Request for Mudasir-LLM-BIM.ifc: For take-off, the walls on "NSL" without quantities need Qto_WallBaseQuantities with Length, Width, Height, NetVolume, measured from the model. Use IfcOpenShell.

First a look at what the model holds.

```python
import ifcopenshell
import ifcopenshell.util.element
import ifcopenshell.util.unit

model = ifcopenshell.open("Mudasir-LLM-BIM.ifc")
print(model.schema)
for unit_type in ("LENGTHUNIT", "AREAUNIT", "VOLUMEUNIT"):
    print(unit_type, ifcopenshell.util.unit.calculate_unit_scale(model, unit_type))
storey = next(s for s in model.by_type("IfcBuildingStorey") if s.Name == "NSL")
walls = [e for e in ifcopenshell.util.element.get_decomposition(storey) if e.is_a("IfcWall")]
for e in sorted(walls, key=lambda e: e.id()):
    print(e.id(), e.is_a(), e.Name, list(ifcopenshell.util.element.get_psets(e, qtos_only=True)), sep=" | ")
```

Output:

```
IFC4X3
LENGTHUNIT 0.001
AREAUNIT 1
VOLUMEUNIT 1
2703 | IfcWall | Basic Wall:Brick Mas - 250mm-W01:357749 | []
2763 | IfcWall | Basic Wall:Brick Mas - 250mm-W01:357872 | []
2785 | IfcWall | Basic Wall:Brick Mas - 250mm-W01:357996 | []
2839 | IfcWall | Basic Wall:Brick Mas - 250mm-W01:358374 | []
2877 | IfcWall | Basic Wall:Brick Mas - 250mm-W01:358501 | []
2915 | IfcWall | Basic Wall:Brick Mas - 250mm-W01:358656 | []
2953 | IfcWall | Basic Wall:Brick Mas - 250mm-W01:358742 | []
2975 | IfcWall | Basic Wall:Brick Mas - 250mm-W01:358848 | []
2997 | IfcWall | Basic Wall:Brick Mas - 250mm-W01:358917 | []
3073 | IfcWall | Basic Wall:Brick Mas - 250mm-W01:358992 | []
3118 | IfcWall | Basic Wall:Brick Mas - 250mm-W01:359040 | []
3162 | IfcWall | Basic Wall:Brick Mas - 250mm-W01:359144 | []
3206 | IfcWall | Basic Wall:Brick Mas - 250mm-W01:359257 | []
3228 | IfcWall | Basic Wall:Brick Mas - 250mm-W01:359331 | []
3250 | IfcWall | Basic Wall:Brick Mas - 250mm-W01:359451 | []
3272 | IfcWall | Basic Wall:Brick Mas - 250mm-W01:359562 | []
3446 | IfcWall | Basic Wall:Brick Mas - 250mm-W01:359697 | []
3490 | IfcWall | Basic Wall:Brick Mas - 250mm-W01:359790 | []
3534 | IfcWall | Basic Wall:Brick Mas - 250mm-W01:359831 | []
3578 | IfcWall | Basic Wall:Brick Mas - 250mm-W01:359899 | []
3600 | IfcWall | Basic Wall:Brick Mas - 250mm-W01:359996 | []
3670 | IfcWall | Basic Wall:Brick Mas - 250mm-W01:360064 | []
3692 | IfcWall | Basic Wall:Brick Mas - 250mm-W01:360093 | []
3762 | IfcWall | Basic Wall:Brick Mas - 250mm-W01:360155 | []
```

```python
import ifcopenshell
import ifcopenshell.api.pset
import ifcopenshell.geom
import ifcopenshell.util.element
import ifcopenshell.util.shape
import ifcopenshell.util.unit

model = ifcopenshell.open("Mudasir-LLM-BIM.ifc")
unit_scale = ifcopenshell.util.unit.calculate_unit_scale(model)
volume_scale = ifcopenshell.util.unit.calculate_unit_scale(model, "VOLUMEUNIT")
settings = ifcopenshell.geom.settings()

storey = next(s for s in model.by_type("IfcBuildingStorey") if s.Name == "NSL")
walls = [e for e in ifcopenshell.util.element.get_decomposition(storey) if e.is_a("IfcWall")]

for e in sorted(walls, key=lambda e: e.id()):
    if ifcopenshell.util.element.get_psets(e, qtos_only=True, should_inherit=False):
        continue
    # Geometry comes back in metres, in the element's own axes.
    shape = ifcopenshell.geom.create_shape(settings, e)
    values = {
        "Length": ifcopenshell.util.shape.get_x(shape.geometry) / unit_scale,
        "Width": ifcopenshell.util.shape.get_y(shape.geometry) / unit_scale,
        "Height": ifcopenshell.util.shape.get_z(shape.geometry) / unit_scale,
        "NetVolume": ifcopenshell.util.shape.get_volume(shape.geometry) / volume_scale,
    }
    qto = ifcopenshell.api.pset.add_qto(model, product=e, name="Qto_WallBaseQuantities")
    ifcopenshell.api.pset.edit_qto(model, qto=qto, properties=values)
    print(e.id(), {k: round(v, 3) for k, v in values.items()})

model.write("Mudasir-LLM-BIM_updated.ifc")
```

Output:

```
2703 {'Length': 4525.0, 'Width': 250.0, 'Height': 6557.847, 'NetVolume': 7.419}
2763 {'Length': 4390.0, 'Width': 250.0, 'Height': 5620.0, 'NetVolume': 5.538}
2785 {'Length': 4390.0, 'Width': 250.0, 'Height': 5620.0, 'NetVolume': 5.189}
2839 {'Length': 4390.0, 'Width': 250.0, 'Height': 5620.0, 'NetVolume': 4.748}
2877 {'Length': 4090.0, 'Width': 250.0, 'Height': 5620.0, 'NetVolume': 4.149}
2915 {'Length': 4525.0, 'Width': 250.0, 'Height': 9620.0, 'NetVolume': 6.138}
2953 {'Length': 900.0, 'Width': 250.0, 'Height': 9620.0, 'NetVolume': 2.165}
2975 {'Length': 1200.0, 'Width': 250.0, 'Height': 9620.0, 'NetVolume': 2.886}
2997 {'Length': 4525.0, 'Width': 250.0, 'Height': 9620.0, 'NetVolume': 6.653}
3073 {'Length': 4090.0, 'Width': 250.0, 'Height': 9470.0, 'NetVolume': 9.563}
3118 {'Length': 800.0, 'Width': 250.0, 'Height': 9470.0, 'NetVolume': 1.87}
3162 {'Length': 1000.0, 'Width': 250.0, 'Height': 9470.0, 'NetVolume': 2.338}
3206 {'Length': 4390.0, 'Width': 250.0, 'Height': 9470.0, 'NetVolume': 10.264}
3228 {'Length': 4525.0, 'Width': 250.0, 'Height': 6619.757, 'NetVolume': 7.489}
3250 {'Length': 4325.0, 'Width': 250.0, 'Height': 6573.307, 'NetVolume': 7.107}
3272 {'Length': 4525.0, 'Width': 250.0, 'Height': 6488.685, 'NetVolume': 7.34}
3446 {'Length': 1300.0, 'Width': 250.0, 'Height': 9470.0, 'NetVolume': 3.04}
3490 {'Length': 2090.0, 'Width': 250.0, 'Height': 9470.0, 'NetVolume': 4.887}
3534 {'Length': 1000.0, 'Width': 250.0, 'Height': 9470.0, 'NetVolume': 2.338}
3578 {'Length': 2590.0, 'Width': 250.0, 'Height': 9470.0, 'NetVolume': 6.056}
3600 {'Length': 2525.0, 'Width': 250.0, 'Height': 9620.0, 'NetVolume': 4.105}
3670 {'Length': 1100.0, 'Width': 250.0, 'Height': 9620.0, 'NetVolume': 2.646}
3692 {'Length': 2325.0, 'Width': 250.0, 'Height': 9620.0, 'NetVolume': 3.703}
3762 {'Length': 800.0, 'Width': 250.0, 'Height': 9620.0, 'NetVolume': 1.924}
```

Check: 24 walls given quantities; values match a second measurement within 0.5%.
